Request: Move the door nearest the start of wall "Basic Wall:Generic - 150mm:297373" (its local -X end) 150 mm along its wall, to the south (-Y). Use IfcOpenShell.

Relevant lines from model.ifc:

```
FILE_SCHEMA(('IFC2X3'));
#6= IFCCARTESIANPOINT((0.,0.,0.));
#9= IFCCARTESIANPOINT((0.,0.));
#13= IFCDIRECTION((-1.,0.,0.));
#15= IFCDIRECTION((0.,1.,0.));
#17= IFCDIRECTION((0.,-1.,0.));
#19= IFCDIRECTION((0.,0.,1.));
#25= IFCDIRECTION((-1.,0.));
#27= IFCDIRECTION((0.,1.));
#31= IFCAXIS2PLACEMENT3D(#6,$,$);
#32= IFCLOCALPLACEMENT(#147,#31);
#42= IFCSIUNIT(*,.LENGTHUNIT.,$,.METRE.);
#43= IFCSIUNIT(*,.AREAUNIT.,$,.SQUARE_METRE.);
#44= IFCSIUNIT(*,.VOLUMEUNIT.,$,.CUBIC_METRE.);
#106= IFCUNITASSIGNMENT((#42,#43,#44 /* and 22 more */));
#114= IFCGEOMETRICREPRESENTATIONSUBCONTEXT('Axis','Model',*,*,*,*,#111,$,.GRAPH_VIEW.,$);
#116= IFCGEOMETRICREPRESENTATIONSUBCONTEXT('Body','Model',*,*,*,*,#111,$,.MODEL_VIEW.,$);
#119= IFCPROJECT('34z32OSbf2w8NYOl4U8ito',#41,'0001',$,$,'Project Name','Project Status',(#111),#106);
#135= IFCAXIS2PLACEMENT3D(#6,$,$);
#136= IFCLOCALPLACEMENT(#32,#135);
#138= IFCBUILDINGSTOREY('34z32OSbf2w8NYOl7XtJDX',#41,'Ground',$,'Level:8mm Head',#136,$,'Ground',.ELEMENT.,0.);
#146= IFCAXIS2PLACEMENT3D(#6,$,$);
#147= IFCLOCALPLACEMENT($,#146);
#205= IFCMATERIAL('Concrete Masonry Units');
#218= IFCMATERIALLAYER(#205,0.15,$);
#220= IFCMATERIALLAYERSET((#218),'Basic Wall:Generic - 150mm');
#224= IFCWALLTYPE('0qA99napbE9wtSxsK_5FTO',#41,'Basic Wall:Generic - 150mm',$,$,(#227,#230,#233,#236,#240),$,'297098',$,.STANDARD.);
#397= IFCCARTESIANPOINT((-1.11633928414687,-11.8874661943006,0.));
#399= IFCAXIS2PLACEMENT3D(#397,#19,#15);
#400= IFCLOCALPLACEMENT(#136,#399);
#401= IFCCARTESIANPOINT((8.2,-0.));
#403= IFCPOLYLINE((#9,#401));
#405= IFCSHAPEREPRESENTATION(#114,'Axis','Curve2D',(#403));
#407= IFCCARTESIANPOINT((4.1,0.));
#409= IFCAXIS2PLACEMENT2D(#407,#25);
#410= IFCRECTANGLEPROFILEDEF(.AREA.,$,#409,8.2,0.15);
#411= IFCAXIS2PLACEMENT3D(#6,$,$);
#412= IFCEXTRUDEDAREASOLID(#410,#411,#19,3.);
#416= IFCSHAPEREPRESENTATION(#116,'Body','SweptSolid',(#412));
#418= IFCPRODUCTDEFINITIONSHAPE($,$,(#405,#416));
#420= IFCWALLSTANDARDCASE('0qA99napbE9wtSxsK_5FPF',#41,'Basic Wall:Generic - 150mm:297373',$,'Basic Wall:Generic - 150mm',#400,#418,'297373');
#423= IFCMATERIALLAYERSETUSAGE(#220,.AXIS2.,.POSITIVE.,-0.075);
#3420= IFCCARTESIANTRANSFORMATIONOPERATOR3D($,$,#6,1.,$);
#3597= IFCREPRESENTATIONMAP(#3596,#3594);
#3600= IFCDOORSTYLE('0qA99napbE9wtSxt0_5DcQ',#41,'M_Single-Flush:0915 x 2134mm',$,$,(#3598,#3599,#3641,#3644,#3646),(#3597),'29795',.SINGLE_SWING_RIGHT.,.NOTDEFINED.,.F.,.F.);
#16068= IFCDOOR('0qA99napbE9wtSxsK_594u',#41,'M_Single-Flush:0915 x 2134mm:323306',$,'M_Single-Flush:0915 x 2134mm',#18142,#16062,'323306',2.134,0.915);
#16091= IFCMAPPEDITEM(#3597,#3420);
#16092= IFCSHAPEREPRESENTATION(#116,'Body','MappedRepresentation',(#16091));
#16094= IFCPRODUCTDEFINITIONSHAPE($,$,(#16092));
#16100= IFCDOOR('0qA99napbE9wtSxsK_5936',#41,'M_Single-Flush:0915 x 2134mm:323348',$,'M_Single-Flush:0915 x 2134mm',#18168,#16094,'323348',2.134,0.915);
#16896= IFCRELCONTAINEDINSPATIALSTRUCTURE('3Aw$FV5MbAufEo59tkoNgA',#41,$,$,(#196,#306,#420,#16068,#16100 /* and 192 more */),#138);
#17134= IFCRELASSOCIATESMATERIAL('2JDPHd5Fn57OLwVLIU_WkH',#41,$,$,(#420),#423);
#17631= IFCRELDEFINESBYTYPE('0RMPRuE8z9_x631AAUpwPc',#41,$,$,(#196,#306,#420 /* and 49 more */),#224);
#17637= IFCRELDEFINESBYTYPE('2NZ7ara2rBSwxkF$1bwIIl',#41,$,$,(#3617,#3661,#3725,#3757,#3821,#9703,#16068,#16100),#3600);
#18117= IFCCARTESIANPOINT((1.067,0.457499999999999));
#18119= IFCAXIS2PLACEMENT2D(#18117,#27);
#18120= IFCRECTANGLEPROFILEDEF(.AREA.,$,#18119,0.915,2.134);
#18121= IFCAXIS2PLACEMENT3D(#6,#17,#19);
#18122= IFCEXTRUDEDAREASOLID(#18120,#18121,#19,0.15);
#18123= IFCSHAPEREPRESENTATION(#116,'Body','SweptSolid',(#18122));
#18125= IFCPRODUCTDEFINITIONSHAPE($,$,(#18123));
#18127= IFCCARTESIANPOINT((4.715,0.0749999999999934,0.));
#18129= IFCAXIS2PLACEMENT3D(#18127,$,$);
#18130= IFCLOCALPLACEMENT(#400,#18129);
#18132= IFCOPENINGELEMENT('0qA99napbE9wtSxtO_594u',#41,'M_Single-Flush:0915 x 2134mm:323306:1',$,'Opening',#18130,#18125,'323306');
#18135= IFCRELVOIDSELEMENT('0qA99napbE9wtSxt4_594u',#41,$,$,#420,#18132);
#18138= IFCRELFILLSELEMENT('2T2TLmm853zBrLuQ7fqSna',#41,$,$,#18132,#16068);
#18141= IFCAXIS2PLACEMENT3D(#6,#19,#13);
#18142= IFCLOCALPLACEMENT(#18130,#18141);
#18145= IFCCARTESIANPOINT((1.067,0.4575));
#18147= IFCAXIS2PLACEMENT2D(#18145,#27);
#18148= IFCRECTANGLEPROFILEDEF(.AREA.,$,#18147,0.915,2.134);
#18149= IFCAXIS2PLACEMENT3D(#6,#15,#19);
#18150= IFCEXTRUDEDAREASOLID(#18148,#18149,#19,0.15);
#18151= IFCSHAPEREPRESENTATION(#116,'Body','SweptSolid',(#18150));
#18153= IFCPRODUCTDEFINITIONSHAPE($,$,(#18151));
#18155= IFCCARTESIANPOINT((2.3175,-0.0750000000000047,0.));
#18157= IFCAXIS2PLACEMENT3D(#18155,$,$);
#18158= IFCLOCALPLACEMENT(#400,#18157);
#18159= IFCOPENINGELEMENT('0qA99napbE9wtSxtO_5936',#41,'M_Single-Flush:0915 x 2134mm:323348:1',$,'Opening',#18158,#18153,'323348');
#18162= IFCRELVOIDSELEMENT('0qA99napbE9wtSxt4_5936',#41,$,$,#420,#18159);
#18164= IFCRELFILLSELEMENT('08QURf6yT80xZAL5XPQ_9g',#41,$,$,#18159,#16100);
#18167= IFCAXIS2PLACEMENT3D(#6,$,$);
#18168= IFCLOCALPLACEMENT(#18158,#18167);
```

```python
import ifcopenshell
import ifcopenshell.api.geometry
import ifcopenshell.util.placement
import ifcopenshell.util.unit

model = ifcopenshell.open("model.ifc")
unit_scale = ifcopenshell.util.unit.calculate_unit_scale(model)

door = model.by_id(16100)
opening = door.FillsVoids[0].RelatingOpeningElement
wall = opening.VoidsElements[0].RelatingBuildingElement

wall_matrix = ifcopenshell.util.placement.get_local_placement(wall.ObjectPlacement)
shift = wall_matrix[:3, 0] * -0.15 / unit_scale
before = ifcopenshell.util.placement.get_local_placement(door.ObjectPlacement)[:3, 3].copy()

# The door is placed relative to its opening, so it follows when the opening moves.
matrix = ifcopenshell.util.placement.get_local_placement(opening.ObjectPlacement)
matrix[:3, 3] += shift
ifcopenshell.api.geometry.edit_object_placement(
    model, product=opening, matrix=matrix, is_si=False, should_transform_children=True
)

after = ifcopenshell.util.placement.get_local_placement(door.ObjectPlacement)[:3, 3]
print("door moved by", (after - before).round(3) + 0.0)

model.write("model_updated.ifc")
```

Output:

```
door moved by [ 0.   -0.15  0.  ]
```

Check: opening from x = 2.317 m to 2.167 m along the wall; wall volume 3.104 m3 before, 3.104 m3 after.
